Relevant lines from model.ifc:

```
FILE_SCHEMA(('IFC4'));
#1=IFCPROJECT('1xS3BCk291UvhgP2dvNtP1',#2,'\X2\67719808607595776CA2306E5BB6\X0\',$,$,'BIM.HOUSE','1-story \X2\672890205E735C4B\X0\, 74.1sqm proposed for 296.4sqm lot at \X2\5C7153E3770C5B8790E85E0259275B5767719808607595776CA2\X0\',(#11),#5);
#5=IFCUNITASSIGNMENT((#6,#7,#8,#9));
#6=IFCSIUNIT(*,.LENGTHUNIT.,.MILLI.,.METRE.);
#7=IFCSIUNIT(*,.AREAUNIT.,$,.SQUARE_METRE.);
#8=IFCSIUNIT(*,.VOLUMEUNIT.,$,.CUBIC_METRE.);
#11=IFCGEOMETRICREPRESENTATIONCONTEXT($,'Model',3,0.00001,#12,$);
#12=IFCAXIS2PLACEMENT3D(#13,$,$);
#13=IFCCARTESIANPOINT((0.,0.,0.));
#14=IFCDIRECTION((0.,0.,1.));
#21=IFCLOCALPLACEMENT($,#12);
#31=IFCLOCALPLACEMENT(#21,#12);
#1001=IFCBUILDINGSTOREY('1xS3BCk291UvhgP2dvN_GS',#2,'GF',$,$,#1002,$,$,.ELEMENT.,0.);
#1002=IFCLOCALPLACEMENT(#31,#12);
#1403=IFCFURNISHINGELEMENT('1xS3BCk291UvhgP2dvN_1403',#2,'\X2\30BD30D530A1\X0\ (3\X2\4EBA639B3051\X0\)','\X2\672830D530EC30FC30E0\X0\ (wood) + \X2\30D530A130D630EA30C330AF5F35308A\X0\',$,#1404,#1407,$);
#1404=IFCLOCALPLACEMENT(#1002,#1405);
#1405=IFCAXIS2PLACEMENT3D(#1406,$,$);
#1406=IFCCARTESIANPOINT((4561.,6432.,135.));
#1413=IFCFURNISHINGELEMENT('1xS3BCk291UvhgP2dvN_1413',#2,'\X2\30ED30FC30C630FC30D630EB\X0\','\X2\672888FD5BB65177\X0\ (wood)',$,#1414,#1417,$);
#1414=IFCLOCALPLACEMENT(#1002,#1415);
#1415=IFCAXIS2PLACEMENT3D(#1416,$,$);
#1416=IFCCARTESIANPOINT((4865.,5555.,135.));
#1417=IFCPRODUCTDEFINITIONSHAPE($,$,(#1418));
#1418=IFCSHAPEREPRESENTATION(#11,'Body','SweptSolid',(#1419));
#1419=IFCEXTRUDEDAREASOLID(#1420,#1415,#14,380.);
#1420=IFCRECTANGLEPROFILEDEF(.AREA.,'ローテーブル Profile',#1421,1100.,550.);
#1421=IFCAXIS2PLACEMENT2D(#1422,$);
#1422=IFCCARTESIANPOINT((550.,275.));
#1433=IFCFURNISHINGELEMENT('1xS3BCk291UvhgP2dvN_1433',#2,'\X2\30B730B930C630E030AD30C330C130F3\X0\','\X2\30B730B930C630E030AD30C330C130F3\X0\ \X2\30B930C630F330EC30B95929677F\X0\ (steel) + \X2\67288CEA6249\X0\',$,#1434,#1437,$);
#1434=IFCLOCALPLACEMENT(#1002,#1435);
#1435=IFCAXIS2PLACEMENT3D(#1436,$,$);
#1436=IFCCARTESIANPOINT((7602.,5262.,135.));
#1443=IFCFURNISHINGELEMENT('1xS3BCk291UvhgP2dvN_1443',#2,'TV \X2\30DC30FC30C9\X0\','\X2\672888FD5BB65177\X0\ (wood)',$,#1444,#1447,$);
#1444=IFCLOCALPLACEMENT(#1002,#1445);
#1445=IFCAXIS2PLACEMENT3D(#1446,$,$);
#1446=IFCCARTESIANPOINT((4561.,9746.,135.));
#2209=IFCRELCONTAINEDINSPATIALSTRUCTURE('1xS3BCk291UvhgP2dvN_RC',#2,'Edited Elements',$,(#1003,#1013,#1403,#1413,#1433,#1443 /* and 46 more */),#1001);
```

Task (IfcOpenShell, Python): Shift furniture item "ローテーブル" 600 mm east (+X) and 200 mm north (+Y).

```python
import ifcopenshell
import ifcopenshell.api.geometry
import ifcopenshell.util.placement

model = ifcopenshell.open("model.ifc")

item = model.by_guid("1xS3BCk291UvhgP2dvN_1413")
matrix = ifcopenshell.util.placement.get_local_placement(item.ObjectPlacement)
matrix[0, 3] += 600.0
matrix[1, 3] += 200.0
ifcopenshell.api.geometry.edit_object_placement(model, product=item, matrix=matrix, is_si=False)

print(ifcopenshell.util.placement.get_local_placement(item.ObjectPlacement).round(3) + 0.0)

model.write("model_edited.ifc")
```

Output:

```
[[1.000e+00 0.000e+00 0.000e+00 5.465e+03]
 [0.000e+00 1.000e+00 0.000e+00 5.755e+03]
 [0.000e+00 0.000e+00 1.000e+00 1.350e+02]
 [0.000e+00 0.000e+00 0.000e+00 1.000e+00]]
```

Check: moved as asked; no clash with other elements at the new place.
